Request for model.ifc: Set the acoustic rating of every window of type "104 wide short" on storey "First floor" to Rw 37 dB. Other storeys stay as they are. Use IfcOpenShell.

First a look at what the model holds.

```python
import ifcopenshell
import ifcopenshell.util.element

model = ifcopenshell.open("model.ifc")
print(model.schema)
storey = next(s for s in model.by_type("IfcBuildingStorey") if s.Name == "First floor")
windows = [e for e in ifcopenshell.util.element.get_decomposition(storey) if e.is_a("IfcWindow")]
seen = {}
for e in windows:
    element_type = ifcopenshell.util.element.get_type(e)
    key = (element_type.Name if element_type != e and element_type else None, ifcopenshell.util.element.get_pset(e, "Pset_WindowCommon", "AcousticRating"))
    seen[key] = seen.get(key, 0) + 1
for (name, value), count in sorted(seen.items(), key=str):
    print(count, "x", name, "|", value)
```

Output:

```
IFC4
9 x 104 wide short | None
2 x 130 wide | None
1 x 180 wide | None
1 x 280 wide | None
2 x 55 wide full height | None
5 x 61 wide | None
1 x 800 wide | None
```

```python
import ifcopenshell
import ifcopenshell.api.pset
import ifcopenshell.util.element

model = ifcopenshell.open("model.ifc")

storey = next(s for s in model.by_type("IfcBuildingStorey") if s.Name == "First floor")
windows = [e for e in ifcopenshell.util.element.get_decomposition(storey) if e.is_a("IfcWindow")]

count = 0
for e in windows:
    element_type = ifcopenshell.util.element.get_type(e)
    if element_type in (None, e) or element_type.Name != "104 wide short":
        continue
    # add_pset returns the element's existing set when there is one.
    pset = ifcopenshell.api.pset.add_pset(model, product=e, name="Pset_WindowCommon")
    ifcopenshell.api.pset.edit_pset(model, pset=pset, properties={"AcousticRating": "Rw 37 dB"})
    count += 1

print(count, "windows updated")

model.write("model_rev.ifc")
```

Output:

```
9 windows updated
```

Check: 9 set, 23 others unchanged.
